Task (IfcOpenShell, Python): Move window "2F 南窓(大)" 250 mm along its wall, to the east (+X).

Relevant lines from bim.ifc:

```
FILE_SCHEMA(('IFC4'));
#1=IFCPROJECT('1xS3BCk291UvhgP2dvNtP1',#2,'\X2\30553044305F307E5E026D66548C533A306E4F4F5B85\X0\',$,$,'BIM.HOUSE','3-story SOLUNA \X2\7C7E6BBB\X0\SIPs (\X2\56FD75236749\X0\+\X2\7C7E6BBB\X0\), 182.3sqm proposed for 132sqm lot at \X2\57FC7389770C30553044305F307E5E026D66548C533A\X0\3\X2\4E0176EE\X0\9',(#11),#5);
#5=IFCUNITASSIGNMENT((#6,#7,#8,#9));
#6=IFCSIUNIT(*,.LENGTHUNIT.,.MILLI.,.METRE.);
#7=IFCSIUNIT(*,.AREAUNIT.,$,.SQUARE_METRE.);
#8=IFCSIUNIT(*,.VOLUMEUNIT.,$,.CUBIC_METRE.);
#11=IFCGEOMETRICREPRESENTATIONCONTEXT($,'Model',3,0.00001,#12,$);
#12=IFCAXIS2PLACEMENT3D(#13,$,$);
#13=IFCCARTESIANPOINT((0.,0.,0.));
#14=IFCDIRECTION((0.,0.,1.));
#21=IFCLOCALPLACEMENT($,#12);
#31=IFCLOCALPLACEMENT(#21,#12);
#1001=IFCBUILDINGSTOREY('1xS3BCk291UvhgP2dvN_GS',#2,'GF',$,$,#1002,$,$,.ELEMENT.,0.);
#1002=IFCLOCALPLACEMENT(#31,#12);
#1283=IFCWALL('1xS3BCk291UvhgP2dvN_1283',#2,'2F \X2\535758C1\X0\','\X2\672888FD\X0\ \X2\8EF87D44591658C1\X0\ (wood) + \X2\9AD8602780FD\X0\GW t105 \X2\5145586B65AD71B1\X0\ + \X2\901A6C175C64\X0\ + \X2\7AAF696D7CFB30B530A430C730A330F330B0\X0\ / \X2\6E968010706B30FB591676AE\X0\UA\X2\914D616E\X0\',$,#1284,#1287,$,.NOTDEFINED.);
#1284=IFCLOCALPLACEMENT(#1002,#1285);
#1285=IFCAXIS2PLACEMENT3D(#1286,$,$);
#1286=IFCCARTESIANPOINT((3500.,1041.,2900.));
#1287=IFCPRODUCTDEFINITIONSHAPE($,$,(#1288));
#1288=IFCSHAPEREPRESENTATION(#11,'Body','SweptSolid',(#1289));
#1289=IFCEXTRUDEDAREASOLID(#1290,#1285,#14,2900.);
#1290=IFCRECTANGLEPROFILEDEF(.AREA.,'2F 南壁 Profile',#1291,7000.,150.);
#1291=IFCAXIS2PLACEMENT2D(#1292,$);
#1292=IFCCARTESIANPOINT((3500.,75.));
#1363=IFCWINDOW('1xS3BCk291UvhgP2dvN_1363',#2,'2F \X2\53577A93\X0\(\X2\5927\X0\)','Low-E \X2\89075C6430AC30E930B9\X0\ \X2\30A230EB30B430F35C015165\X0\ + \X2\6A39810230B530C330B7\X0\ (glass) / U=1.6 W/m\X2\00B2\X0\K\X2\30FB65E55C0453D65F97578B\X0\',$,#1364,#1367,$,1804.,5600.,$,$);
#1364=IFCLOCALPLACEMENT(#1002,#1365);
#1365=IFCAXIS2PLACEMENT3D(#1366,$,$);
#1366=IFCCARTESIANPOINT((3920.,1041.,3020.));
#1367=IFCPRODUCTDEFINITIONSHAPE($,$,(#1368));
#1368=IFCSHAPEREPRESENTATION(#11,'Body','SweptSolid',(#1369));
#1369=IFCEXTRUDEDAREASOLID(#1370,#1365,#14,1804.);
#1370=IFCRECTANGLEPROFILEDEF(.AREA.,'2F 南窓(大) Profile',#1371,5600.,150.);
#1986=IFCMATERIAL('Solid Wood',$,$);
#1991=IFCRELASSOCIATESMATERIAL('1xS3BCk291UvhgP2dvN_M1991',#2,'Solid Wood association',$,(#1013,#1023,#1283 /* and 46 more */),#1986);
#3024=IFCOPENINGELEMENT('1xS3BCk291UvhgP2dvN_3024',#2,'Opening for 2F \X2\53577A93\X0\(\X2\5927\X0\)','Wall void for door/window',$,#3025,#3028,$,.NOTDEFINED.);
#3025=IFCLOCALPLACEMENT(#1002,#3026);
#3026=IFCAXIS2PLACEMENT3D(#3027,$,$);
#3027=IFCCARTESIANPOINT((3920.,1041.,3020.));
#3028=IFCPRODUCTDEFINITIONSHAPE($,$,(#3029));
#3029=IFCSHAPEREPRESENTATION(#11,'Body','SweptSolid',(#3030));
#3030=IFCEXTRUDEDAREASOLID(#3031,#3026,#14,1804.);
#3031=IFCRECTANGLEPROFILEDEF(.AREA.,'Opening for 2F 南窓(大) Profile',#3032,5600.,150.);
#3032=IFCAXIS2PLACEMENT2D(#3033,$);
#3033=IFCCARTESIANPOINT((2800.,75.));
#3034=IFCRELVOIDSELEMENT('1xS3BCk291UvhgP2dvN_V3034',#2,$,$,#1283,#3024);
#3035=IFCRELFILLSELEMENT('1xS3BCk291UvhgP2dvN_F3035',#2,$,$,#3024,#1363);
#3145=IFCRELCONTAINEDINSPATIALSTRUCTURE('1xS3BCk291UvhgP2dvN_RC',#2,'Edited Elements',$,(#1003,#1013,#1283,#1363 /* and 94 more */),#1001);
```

```python
import ifcopenshell
import ifcopenshell.api.geometry
import ifcopenshell.util.placement
import ifcopenshell.util.unit

model = ifcopenshell.open("bim.ifc")
unit_scale = ifcopenshell.util.unit.calculate_unit_scale(model)

window = model.by_id(1363)
opening = window.FillsVoids[0].RelatingOpeningElement
wall = opening.VoidsElements[0].RelatingBuildingElement

wall_matrix = ifcopenshell.util.placement.get_local_placement(wall.ObjectPlacement)
shift = wall_matrix[:3, 0] * 0.25 / unit_scale
before = ifcopenshell.util.placement.get_local_placement(window.ObjectPlacement)[:3, 3].copy()

# The window is not placed relative to its opening, so move both.
for product in (opening, window):
    matrix = ifcopenshell.util.placement.get_local_placement(product.ObjectPlacement)
    matrix[:3, 3] += shift
    ifcopenshell.api.geometry.edit_object_placement(model, product=product, matrix=matrix, is_si=False)

after = ifcopenshell.util.placement.get_local_placement(window.ObjectPlacement)[:3, 3]
print("window moved by", (after - before).round(3) + 0.0)

model.write("bim_v2.ifc")
```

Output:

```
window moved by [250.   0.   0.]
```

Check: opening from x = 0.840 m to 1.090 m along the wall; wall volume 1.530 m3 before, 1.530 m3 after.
